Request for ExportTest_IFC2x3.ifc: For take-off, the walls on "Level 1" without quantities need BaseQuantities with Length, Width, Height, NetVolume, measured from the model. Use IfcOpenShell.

First a look at what the model holds.

```python
import ifcopenshell
import ifcopenshell.util.element
import ifcopenshell.util.unit

model = ifcopenshell.open("ExportTest_IFC2x3.ifc")
print(model.schema)
for unit_type in ("LENGTHUNIT", "AREAUNIT", "VOLUMEUNIT"):
    print(unit_type, ifcopenshell.util.unit.calculate_unit_scale(model, unit_type))
storey = next(s for s in model.by_type("IfcBuildingStorey") if s.Name == "Level 1")
walls = [e for e in ifcopenshell.util.element.get_decomposition(storey) if e.is_a("IfcWall")]
for e in sorted(walls, key=lambda e: e.id()):
    print(e.id(), e.is_a(), e.Name, list(ifcopenshell.util.element.get_psets(e, qtos_only=True)), sep=" | ")
```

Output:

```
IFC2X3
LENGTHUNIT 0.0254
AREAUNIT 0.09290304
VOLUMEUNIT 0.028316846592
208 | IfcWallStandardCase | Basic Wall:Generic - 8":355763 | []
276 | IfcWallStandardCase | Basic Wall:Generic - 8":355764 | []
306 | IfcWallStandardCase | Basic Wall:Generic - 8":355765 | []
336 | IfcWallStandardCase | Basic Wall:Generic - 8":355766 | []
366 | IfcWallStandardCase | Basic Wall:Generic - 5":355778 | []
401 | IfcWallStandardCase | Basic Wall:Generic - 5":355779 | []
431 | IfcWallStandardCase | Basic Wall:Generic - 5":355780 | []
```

```python
import ifcopenshell
import ifcopenshell.api.pset
import ifcopenshell.geom
import ifcopenshell.util.element
import ifcopenshell.util.shape
import ifcopenshell.util.unit

model = ifcopenshell.open("ExportTest_IFC2x3.ifc")
unit_scale = ifcopenshell.util.unit.calculate_unit_scale(model)
volume_scale = ifcopenshell.util.unit.calculate_unit_scale(model, "VOLUMEUNIT")
settings = ifcopenshell.geom.settings()

storey = next(s for s in model.by_type("IfcBuildingStorey") if s.Name == "Level 1")
walls = [e for e in ifcopenshell.util.element.get_decomposition(storey) if e.is_a("IfcWall")]

for e in sorted(walls, key=lambda e: e.id()):
    if ifcopenshell.util.element.get_psets(e, qtos_only=True, should_inherit=False):
        continue
    # Geometry comes back in metres, in the element's own axes.
    shape = ifcopenshell.geom.create_shape(settings, e)
    values = {
        "Length": ifcopenshell.util.shape.get_x(shape.geometry) / unit_scale,
        "Width": ifcopenshell.util.shape.get_y(shape.geometry) / unit_scale,
        "Height": ifcopenshell.util.shape.get_z(shape.geometry) / unit_scale,
        "NetVolume": ifcopenshell.util.shape.get_volume(shape.geometry) / volume_scale,
    }
    qto = ifcopenshell.api.pset.add_qto(model, product=e, name="BaseQuantities")
    ifcopenshell.api.pset.edit_qto(model, qto=qto, properties=values)
    print(e.id(), {k: round(v, 3) for k, v in values.items()})

model.write("ExportTest_IFC2x3_rev.ifc")
```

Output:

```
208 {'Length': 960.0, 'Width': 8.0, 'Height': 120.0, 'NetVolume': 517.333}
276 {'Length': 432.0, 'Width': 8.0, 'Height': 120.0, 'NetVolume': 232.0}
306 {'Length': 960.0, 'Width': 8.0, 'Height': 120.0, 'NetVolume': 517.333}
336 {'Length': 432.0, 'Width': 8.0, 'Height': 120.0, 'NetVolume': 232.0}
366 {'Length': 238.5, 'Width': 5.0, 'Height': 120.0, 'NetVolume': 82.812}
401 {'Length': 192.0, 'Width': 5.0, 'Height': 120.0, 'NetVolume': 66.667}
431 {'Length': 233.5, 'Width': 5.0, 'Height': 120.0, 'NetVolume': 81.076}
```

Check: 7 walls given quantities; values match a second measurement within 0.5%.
